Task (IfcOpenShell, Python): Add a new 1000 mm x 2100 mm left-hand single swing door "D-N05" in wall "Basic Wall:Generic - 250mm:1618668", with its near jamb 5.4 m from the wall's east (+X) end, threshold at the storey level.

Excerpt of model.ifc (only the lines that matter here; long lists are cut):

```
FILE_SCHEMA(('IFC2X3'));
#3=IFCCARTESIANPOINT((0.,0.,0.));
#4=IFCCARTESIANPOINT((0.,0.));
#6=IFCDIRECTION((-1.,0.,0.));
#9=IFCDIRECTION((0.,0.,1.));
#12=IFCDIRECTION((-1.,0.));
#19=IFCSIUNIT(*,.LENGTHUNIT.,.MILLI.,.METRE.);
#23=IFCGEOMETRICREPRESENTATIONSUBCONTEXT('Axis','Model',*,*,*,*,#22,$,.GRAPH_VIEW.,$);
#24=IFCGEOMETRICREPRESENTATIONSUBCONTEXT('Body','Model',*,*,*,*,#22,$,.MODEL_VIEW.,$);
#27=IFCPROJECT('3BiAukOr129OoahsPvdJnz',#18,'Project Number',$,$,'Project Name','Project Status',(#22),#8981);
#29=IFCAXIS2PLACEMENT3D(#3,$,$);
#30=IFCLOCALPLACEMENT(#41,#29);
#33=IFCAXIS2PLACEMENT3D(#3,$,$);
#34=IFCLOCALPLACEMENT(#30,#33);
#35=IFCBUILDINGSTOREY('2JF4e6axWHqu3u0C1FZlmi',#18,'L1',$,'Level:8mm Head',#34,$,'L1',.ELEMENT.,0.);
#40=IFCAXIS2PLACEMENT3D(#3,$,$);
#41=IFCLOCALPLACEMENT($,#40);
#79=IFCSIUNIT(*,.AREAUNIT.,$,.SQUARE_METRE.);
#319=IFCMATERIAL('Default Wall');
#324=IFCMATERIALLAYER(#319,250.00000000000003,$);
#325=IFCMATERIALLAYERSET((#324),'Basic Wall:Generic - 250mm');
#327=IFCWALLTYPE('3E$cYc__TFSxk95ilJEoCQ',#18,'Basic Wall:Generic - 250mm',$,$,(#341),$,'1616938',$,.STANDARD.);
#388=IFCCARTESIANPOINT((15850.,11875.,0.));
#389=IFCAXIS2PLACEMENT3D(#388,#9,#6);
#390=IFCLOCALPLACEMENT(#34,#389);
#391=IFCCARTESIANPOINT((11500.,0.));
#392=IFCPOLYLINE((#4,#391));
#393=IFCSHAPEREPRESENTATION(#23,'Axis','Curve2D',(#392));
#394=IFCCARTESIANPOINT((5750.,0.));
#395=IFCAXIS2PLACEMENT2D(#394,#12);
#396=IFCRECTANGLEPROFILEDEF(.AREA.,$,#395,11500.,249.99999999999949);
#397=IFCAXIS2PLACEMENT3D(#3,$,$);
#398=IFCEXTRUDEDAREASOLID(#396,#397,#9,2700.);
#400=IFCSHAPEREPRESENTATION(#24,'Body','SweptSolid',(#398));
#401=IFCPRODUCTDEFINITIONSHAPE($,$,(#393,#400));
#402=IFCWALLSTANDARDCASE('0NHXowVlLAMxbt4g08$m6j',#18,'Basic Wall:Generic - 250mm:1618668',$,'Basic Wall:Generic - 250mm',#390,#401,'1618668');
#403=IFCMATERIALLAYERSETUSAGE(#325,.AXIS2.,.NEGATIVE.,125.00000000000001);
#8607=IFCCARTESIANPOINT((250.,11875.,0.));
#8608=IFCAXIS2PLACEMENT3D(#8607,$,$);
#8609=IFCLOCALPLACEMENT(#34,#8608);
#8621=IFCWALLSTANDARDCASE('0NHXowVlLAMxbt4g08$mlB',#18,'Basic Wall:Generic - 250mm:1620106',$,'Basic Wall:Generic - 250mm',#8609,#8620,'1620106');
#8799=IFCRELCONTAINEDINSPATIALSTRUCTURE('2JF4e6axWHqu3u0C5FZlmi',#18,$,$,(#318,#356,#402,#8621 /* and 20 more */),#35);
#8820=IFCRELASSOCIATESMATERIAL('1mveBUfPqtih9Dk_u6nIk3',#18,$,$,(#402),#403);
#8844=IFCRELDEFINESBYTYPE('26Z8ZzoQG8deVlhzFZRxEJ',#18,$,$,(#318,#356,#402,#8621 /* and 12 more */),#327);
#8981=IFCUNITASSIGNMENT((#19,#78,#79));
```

```python
import numpy as np
import ifcopenshell
import ifcopenshell.api.feature
import ifcopenshell.api.geometry
import ifcopenshell.api.root
import ifcopenshell.api.spatial
import ifcopenshell.api.type
import ifcopenshell.geom
import ifcopenshell.util.element
import ifcopenshell.util.placement
import ifcopenshell.util.representation
import ifcopenshell.util.shape
import ifcopenshell.util.unit

model = ifcopenshell.open("model.ifc")
unit_scale = ifcopenshell.util.unit.calculate_unit_scale(model)
settings = ifcopenshell.geom.settings()


def volume(element):
    """Net volume in cubic metres, openings subtracted."""
    shape = ifcopenshell.geom.create_shape(settings, element)
    return ifcopenshell.util.shape.get_volume(shape.geometry)


wall = model.by_guid("0NHXowVlLAMxbt4g08$m6j")
storey = ifcopenshell.util.element.get_container(wall, ifc_class="IfcBuildingStorey")
context = ifcopenshell.util.representation.get_context(model, "Model", "Body", "MODEL_VIEW")
before = volume(wall)

width, height, from_end, sill = 1, 2.1, 5.4, 0.0  # metres

# The wall runs along its own X axis, and the end named is its -X end.
wall_shape = ifcopenshell.geom.create_shape(settings, wall)
x, y, z = ifcopenshell.util.shape.get_vertices(wall_shape.geometry).T
start = x.min() + from_end
face, thickness = float(y.min()), float(y.max() - y.min())
wall_matrix = ifcopenshell.util.placement.get_local_placement(wall.ObjectPlacement)
level = ifcopenshell.util.placement.get_local_placement(storey.ObjectPlacement)[2, 3]


def in_wall(x, y):
    """Placement at x, y metres in the wall's axes, at sill height."""
    matrix = wall_matrix.copy()
    matrix[:, 3] = wall_matrix @ np.array([x / unit_scale, y / unit_scale, 0.0, 1.0])
    matrix[2, 3] = level + sill / unit_scale
    return matrix


# Opening: a box that overshoots both wall faces by 50 mm.
opening = ifcopenshell.api.root.create_entity(model, ifc_class="IfcOpeningElement")
box = ifcopenshell.api.geometry.add_wall_representation(
    model, context=context, length=width, height=height, thickness=thickness + 0.1
)
ifcopenshell.api.geometry.assign_representation(model, product=opening, representation=box)
ifcopenshell.api.geometry.edit_object_placement(model, product=opening, matrix=in_wall(start, face - 0.05), is_si=False)
ifcopenshell.api.feature.add_feature(model, feature=opening, element=wall)

door = ifcopenshell.api.root.create_entity(model, ifc_class="IfcDoor", name="D-N05")
door.OverallWidth, door.OverallHeight = width / unit_scale, height / unit_scale
body = ifcopenshell.api.geometry.add_door_representation(
    model,
    context=context,
    overall_width=door.OverallWidth,
    overall_height=door.OverallHeight,
    operation_type="SINGLE_SWING_LEFT",
    lining_properties={"LiningDepth": thickness / unit_scale, "ThresholdDepth": thickness / unit_scale},
)
ifcopenshell.api.geometry.assign_representation(model, product=door, representation=body)
ifcopenshell.api.spatial.assign_container(model, products=[door], relating_structure=storey)
fills = ifcopenshell.api.feature.add_filling(model, opening=opening, element=door)
fills.OwnerHistory = door.OwnerHistory  # required in IFC2X3

# IFC2X3 keeps the operation on the door style.
style = ifcopenshell.api.root.create_entity(model, ifc_class="IfcDoorStyle", name="D-N05")
style.OperationType, style.ConstructionType = "SINGLE_SWING_LEFT", "NOTDEFINED"
style.ParameterTakesPrecedence = style.Sizeable = False
ifcopenshell.api.type.assign_type(model, related_objects=[door], relating_type=style)

# The lining spans the wall, so the door starts at the wall face.
ifcopenshell.api.geometry.edit_object_placement(model, product=door, matrix=in_wall(start, face), is_si=False)

after = volume(wall)

print(f"wall volume {before:.3f} -> {after:.3f} m3")

model.write("model_rev.ifc")
```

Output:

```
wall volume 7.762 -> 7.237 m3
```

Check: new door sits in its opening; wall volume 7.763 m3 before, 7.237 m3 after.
